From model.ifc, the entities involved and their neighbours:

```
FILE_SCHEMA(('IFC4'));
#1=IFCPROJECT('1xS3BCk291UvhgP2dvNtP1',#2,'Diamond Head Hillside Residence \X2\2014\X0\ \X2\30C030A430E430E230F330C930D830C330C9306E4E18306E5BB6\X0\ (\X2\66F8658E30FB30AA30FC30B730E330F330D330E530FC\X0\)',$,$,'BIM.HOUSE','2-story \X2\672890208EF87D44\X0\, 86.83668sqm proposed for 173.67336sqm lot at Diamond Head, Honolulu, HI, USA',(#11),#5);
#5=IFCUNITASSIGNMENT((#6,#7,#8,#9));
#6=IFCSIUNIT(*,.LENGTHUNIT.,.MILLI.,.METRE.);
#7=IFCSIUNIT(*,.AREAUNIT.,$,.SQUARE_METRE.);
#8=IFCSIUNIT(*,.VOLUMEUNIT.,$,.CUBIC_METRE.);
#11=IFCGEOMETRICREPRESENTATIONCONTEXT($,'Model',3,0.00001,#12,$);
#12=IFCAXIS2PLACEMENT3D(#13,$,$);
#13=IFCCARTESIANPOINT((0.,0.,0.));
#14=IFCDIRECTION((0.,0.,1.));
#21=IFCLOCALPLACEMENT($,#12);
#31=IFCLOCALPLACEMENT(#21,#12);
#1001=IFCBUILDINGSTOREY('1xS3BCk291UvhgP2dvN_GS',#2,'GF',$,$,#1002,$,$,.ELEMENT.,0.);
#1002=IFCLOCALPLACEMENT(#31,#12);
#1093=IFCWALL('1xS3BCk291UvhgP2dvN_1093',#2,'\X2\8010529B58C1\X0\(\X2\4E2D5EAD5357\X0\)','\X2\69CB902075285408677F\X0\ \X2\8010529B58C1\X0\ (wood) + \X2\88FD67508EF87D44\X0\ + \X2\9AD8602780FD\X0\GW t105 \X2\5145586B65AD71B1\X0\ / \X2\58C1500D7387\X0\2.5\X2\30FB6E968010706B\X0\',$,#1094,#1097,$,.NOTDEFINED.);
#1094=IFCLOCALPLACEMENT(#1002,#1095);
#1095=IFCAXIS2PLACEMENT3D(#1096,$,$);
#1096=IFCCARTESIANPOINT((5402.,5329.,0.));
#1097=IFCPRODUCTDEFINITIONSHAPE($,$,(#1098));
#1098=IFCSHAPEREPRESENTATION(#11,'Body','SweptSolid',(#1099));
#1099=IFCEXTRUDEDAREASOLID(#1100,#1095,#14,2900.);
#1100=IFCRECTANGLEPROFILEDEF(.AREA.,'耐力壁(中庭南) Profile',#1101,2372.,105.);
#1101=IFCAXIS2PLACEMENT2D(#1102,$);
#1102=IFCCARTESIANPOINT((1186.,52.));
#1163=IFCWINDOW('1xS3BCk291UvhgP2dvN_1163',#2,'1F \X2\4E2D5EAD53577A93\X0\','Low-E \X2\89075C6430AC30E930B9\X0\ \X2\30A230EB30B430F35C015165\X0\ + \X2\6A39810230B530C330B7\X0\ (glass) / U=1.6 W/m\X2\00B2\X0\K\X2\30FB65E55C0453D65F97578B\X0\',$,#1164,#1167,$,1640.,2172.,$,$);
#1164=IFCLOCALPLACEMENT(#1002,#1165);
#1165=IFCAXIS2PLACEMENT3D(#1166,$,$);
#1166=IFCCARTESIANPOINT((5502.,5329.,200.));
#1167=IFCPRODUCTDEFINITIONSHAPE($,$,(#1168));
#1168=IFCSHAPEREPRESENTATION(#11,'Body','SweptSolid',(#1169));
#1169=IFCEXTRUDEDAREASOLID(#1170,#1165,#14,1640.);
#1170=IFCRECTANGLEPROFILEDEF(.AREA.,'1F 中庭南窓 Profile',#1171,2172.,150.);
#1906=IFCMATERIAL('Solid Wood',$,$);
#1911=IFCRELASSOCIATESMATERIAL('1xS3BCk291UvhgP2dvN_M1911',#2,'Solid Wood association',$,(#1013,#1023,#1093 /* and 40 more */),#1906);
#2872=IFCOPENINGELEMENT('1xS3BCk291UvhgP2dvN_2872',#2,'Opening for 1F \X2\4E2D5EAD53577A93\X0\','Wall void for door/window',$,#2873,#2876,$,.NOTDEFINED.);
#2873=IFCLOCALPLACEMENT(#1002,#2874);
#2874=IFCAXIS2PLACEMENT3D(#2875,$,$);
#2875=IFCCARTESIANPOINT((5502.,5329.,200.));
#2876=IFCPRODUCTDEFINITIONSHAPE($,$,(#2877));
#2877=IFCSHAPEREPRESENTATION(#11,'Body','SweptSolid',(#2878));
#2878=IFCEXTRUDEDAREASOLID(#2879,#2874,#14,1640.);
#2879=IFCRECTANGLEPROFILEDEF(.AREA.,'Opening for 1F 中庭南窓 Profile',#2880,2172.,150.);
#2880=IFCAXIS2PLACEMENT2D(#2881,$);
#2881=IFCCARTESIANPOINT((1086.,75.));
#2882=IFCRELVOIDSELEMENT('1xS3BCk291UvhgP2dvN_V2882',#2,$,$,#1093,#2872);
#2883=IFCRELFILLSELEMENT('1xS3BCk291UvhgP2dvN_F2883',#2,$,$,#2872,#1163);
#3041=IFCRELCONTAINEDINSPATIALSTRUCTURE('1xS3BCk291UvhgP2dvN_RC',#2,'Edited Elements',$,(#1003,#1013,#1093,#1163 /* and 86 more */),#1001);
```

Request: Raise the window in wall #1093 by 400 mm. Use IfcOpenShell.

```python
import numpy as np
import ifcopenshell
import ifcopenshell.api.geometry
import ifcopenshell.util.placement
import ifcopenshell.util.unit

model = ifcopenshell.open("model.ifc")
unit_scale = ifcopenshell.util.unit.calculate_unit_scale(model)

window = model.by_id(1163)
opening = window.FillsVoids[0].RelatingOpeningElement
dz = 400.0

shift = np.array([0.0, 0.0, dz])
# The window is not placed relative to its opening, so move both.
for product in (opening, window):
    matrix = ifcopenshell.util.placement.get_local_placement(product.ObjectPlacement)
    matrix[:3, 3] += shift
    ifcopenshell.api.geometry.edit_object_placement(model, product=product, matrix=matrix, is_si=False)

print(f"moved by {dz * unit_scale:+.3f} m")

model.write("model_updated.ifc")
```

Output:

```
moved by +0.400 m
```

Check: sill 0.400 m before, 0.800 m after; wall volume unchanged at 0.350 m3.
